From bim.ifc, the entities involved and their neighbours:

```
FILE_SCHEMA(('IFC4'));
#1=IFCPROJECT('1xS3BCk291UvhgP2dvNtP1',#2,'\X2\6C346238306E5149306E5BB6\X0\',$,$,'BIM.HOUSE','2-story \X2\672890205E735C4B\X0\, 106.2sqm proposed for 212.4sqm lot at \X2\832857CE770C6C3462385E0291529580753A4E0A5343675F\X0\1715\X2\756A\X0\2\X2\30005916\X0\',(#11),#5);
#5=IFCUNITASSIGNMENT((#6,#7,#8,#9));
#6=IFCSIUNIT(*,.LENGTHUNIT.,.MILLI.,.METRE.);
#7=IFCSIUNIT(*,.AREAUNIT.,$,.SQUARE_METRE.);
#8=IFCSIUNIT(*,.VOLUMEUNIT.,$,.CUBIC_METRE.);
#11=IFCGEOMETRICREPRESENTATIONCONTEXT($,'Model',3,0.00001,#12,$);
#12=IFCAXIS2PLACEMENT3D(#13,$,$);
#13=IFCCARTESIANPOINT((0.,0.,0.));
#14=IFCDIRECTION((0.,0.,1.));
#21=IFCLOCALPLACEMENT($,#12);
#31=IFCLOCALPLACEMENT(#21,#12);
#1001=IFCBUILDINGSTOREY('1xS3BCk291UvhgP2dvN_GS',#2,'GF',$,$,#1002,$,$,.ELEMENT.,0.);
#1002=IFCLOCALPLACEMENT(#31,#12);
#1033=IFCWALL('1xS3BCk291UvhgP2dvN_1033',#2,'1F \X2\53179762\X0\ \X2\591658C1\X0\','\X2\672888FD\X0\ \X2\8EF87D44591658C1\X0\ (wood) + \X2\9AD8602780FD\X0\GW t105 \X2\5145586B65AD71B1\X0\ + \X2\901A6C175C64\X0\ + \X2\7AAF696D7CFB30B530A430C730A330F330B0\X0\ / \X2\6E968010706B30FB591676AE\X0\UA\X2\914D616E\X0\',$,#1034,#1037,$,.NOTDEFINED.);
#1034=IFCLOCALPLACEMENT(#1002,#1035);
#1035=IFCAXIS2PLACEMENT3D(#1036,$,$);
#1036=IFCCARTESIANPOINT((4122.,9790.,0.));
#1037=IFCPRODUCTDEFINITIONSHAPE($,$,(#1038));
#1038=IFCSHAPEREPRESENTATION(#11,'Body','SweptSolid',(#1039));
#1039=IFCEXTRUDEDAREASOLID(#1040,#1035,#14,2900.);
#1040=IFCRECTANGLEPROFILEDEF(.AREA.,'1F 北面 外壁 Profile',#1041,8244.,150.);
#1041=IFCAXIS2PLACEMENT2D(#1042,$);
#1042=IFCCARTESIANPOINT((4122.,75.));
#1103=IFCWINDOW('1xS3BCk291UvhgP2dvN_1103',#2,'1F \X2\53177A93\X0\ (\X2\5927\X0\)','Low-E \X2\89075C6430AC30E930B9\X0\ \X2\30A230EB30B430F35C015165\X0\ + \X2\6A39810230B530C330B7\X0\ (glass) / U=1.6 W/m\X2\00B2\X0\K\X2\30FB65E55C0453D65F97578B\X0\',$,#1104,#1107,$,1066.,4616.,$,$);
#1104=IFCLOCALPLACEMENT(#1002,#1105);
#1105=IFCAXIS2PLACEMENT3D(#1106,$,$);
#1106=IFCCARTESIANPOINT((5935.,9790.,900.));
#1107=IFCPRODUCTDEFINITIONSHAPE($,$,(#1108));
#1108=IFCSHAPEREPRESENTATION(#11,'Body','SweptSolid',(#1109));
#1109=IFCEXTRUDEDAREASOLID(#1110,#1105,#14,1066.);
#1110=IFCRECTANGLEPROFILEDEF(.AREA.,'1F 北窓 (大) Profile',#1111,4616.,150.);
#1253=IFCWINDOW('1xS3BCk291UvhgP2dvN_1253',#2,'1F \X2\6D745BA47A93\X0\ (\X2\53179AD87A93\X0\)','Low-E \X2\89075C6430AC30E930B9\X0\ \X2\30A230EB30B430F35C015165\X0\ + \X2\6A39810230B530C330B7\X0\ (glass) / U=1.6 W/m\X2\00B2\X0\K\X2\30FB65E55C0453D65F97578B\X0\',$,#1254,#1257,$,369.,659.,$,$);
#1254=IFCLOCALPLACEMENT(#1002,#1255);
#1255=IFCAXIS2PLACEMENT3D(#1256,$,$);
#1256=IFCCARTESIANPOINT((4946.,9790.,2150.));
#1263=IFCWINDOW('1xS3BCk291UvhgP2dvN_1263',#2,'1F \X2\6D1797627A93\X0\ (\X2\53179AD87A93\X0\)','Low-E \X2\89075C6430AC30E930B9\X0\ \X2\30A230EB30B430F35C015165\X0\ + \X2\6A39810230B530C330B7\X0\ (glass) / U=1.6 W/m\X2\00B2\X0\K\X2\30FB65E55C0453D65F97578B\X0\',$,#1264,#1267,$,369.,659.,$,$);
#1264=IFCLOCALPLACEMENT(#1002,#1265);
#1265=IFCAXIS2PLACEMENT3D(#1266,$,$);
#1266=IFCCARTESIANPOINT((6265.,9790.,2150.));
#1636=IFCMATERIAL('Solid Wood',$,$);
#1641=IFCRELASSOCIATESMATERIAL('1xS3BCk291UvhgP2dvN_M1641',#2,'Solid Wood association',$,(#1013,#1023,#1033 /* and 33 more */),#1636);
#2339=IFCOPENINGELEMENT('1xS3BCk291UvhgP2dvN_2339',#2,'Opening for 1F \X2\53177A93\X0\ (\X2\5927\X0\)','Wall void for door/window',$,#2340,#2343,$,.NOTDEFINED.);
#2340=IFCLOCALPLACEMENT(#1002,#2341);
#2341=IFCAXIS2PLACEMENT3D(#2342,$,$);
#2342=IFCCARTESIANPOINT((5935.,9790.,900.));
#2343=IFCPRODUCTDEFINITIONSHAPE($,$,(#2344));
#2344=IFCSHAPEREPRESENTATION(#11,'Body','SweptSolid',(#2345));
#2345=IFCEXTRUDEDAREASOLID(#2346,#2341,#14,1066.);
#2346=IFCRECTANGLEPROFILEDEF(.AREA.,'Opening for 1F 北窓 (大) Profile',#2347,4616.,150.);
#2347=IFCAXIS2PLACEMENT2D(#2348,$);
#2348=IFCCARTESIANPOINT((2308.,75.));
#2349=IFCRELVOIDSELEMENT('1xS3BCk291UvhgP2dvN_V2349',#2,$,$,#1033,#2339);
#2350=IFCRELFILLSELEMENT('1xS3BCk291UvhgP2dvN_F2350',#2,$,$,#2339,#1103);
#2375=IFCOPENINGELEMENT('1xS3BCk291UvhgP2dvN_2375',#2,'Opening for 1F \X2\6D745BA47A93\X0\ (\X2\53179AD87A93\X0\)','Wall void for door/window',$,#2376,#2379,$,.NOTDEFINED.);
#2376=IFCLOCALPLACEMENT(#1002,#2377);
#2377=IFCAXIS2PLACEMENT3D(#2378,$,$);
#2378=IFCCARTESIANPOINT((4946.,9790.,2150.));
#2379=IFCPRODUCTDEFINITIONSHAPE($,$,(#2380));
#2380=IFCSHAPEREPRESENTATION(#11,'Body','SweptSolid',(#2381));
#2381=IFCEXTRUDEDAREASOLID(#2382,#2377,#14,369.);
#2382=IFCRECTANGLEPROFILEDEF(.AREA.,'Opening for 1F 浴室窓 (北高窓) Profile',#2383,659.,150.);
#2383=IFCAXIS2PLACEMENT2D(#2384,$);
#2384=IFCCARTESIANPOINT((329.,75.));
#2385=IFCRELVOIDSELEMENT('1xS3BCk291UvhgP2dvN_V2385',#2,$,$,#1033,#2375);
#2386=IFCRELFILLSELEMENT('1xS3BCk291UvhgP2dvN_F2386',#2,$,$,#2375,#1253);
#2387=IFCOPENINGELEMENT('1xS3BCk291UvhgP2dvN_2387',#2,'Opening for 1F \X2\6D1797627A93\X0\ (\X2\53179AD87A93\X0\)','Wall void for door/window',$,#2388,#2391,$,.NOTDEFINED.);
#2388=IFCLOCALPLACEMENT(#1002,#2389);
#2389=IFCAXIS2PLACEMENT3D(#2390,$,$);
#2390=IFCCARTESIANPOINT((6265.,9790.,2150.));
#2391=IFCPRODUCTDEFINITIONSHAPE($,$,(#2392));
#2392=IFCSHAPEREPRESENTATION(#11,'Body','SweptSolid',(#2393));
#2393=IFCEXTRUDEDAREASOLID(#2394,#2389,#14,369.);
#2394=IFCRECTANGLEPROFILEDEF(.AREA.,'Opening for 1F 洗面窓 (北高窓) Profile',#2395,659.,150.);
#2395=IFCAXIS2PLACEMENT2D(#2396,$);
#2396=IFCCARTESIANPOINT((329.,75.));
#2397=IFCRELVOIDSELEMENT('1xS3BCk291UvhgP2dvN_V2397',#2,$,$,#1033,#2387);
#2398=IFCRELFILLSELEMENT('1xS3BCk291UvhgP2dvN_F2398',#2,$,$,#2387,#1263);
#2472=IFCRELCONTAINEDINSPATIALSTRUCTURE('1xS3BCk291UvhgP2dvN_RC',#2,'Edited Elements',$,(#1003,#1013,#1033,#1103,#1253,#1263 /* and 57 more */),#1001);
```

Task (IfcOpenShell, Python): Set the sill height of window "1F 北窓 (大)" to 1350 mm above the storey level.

```python
import numpy as np
import ifcopenshell
import ifcopenshell.api.geometry
import ifcopenshell.geom
import ifcopenshell.util.element
import ifcopenshell.util.placement
import ifcopenshell.util.shape
import ifcopenshell.util.unit

model = ifcopenshell.open("bim.ifc")
unit_scale = ifcopenshell.util.unit.calculate_unit_scale(model)

window = model.by_guid("1xS3BCk291UvhgP2dvN_1103")
opening = window.FillsVoids[0].RelatingOpeningElement
storey = ifcopenshell.util.element.get_container(window, ifc_class="IfcBuildingStorey")
level = ifcopenshell.util.placement.get_local_placement(storey.ObjectPlacement)[2, 3]

# The opening's origin need not be at the sill, so measure its lowest point.
shape = ifcopenshell.geom.create_shape(ifcopenshell.geom.settings(), opening)
bottom = ifcopenshell.util.shape.get_shape_bottom_elevation(shape, shape.geometry) / unit_scale
dz = level + 1350.0 - bottom

shift = np.array([0.0, 0.0, dz])
# The window is not placed relative to its opening, so move both.
for product in (opening, window):
    matrix = ifcopenshell.util.placement.get_local_placement(product.ObjectPlacement)
    matrix[:3, 3] += shift
    ifcopenshell.api.geometry.edit_object_placement(model, product=product, matrix=matrix, is_si=False)

print(f"moved by {dz * unit_scale:+.3f} m")

model.write("bim-out.ifc")
```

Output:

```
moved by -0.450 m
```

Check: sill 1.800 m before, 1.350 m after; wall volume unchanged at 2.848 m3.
